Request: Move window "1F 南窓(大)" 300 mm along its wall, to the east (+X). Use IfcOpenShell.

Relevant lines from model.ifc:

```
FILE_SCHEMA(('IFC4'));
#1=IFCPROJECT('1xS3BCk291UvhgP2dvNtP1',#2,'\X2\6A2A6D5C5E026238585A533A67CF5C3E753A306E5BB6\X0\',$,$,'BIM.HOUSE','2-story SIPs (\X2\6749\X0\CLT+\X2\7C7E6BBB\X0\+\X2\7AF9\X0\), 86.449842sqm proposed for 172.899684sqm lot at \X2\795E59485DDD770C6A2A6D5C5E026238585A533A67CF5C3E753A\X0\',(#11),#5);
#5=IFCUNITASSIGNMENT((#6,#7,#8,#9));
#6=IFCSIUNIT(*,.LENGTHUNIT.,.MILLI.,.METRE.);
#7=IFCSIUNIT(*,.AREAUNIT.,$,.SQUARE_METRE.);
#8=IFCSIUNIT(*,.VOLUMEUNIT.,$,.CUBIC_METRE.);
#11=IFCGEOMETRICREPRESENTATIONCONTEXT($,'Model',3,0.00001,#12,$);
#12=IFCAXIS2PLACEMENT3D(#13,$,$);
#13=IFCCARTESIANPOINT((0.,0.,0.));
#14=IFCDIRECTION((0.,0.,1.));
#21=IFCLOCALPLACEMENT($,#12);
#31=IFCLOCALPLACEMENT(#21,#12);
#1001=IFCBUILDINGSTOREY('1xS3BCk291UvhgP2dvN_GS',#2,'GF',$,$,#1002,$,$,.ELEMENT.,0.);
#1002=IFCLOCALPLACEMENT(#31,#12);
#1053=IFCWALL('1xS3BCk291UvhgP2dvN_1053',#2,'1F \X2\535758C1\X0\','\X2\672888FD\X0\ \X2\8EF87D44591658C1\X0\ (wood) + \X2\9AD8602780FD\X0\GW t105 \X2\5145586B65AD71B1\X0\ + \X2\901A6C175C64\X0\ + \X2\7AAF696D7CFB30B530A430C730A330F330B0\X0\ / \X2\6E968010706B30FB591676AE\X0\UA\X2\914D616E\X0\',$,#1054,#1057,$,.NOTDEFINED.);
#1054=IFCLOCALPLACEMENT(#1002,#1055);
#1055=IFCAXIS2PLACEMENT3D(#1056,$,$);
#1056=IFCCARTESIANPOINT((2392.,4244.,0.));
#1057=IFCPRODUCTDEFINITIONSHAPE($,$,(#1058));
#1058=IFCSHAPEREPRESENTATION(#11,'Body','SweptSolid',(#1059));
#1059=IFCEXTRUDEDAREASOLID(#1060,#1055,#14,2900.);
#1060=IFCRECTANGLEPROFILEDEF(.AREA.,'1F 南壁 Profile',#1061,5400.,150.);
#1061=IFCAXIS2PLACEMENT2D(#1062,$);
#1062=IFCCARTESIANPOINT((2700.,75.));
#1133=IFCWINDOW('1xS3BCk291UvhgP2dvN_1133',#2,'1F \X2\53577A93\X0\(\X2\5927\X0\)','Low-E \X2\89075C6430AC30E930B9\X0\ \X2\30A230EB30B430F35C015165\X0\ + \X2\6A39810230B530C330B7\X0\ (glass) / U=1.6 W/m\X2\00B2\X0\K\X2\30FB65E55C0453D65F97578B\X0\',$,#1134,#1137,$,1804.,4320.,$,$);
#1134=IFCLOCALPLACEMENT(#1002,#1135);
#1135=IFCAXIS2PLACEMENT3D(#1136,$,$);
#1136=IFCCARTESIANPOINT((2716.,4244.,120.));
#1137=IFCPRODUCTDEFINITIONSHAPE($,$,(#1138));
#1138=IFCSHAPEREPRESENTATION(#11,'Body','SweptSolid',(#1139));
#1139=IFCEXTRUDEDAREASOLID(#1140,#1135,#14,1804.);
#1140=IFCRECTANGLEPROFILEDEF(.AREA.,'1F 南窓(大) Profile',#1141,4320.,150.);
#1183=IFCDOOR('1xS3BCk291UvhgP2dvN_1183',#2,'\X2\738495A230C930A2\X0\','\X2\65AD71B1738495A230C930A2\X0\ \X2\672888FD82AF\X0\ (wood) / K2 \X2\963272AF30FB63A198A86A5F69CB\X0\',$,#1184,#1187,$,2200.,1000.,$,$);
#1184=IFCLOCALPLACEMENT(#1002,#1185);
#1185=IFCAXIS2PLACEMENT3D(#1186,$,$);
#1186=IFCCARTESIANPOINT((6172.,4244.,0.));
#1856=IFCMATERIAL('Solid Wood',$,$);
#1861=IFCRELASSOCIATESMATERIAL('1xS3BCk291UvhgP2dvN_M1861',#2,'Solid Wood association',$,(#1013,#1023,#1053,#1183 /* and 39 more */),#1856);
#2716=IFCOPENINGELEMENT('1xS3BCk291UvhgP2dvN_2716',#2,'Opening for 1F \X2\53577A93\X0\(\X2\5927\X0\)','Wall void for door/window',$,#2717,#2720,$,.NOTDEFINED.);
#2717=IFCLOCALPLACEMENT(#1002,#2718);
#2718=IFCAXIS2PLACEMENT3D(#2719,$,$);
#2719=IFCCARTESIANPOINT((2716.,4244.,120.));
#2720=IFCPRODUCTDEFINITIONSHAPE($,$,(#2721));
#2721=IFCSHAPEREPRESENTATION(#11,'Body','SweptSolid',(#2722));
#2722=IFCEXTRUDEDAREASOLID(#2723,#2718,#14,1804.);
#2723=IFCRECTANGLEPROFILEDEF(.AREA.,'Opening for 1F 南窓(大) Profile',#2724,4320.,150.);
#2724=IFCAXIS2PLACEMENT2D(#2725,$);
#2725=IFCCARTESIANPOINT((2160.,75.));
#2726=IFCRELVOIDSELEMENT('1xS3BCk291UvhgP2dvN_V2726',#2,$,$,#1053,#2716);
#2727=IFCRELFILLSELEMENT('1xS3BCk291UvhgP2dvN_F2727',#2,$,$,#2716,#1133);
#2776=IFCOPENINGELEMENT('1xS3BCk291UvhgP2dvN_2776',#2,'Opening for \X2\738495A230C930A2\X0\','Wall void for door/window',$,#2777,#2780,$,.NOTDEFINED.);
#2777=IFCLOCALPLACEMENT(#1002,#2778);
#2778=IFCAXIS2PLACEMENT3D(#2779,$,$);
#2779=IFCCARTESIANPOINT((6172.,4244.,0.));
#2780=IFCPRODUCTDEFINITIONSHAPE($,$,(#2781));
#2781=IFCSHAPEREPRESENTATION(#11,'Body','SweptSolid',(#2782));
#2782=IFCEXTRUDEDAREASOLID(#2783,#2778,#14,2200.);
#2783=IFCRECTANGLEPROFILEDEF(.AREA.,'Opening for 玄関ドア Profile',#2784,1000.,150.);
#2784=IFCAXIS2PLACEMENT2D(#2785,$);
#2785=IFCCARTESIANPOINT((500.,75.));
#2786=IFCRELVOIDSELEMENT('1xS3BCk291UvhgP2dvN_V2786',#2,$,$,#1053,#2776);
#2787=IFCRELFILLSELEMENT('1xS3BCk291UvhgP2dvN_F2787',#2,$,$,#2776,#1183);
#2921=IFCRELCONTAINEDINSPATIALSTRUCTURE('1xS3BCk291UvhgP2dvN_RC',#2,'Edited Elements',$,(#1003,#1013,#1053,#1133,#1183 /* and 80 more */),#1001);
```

```python
import ifcopenshell
import ifcopenshell.api.geometry
import ifcopenshell.util.placement
import ifcopenshell.util.unit

model = ifcopenshell.open("model.ifc")
unit_scale = ifcopenshell.util.unit.calculate_unit_scale(model)

window = model.by_id(1133)
opening = window.FillsVoids[0].RelatingOpeningElement
wall = opening.VoidsElements[0].RelatingBuildingElement

wall_matrix = ifcopenshell.util.placement.get_local_placement(wall.ObjectPlacement)
shift = wall_matrix[:3, 0] * 0.3 / unit_scale
before = ifcopenshell.util.placement.get_local_placement(window.ObjectPlacement)[:3, 3].copy()

# The window is not placed relative to its opening, so move both.
for product in (opening, window):
    matrix = ifcopenshell.util.placement.get_local_placement(product.ObjectPlacement)
    matrix[:3, 3] += shift
    ifcopenshell.api.geometry.edit_object_placement(model, product=product, matrix=matrix, is_si=False)

after = ifcopenshell.util.placement.get_local_placement(window.ObjectPlacement)[:3, 3]
print("window moved by", (after - before).round(3) + 0.0)

model.write("model_v2.ifc")
```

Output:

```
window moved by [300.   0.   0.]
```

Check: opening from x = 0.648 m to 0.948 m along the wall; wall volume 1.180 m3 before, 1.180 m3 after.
